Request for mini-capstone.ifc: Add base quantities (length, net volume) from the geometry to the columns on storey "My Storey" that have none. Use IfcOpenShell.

First a look at what the model holds.

```python
import ifcopenshell
import ifcopenshell.util.element
import ifcopenshell.util.unit

model = ifcopenshell.open("mini-capstone.ifc")
print(model.schema)
for unit_type in ("LENGTHUNIT", "AREAUNIT", "VOLUMEUNIT"):
    print(unit_type, ifcopenshell.util.unit.calculate_unit_scale(model, unit_type))
storey = next(s for s in model.by_type("IfcBuildingStorey") if s.Name == "My Storey")
columns = [e for e in ifcopenshell.util.element.get_decomposition(storey) if e.is_a("IfcColumn")]
for e in sorted(columns, key=lambda e: e.id()):
    print(e.id(), e.is_a(), e.Name, list(ifcopenshell.util.element.get_psets(e, qtos_only=True)), sep=" | ")
```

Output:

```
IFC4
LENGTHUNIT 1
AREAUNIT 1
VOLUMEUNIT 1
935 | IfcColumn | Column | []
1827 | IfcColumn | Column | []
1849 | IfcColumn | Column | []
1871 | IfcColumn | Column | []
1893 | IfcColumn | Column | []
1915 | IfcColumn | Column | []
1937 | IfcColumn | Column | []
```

```python
import ifcopenshell
import ifcopenshell.api.pset
import ifcopenshell.geom
import ifcopenshell.util.element
import ifcopenshell.util.shape
import ifcopenshell.util.unit

model = ifcopenshell.open("mini-capstone.ifc")
unit_scale = ifcopenshell.util.unit.calculate_unit_scale(model)
volume_scale = ifcopenshell.util.unit.calculate_unit_scale(model, "VOLUMEUNIT")
settings = ifcopenshell.geom.settings()

storey = next(s for s in model.by_type("IfcBuildingStorey") if s.Name == "My Storey")
columns = [e for e in ifcopenshell.util.element.get_decomposition(storey) if e.is_a("IfcColumn")]

for e in sorted(columns, key=lambda e: e.id()):
    if ifcopenshell.util.element.get_psets(e, qtos_only=True, should_inherit=False):
        continue
    # Geometry comes back in metres, in the element's own axes.
    shape = ifcopenshell.geom.create_shape(settings, e)
    values = {
        "Length": ifcopenshell.util.shape.get_z(shape.geometry) / unit_scale,
        "NetVolume": ifcopenshell.util.shape.get_volume(shape.geometry) / volume_scale,
    }
    qto = ifcopenshell.api.pset.add_qto(model, product=e, name="Qto_ColumnBaseQuantities")
    ifcopenshell.api.pset.edit_qto(model, qto=qto, properties=values)
    print(e.id(), {k: round(v, 3) for k, v in values.items()})

model.write("mini-capstone_rev.ifc")
```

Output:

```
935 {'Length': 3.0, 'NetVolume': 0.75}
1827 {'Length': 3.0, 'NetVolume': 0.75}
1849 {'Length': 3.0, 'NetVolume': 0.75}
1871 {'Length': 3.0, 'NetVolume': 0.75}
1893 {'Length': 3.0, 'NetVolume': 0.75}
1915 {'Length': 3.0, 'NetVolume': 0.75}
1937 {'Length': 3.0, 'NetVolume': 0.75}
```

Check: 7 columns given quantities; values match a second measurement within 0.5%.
